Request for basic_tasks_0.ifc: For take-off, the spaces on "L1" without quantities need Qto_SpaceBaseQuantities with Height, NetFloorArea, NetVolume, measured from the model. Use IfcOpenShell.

First a look at what the model holds.

```python
import ifcopenshell
import ifcopenshell.util.element
import ifcopenshell.util.unit

model = ifcopenshell.open("basic_tasks_0.ifc")
print(model.schema)
for unit_type in ("LENGTHUNIT", "AREAUNIT", "VOLUMEUNIT"):
    print(unit_type, ifcopenshell.util.unit.calculate_unit_scale(model, unit_type))
storey = next(s for s in model.by_type("IfcBuildingStorey") if s.Name == "L1")
spaces = [e for e in ifcopenshell.util.element.get_decomposition(storey) if e.is_a("IfcSpace")]
for e in sorted(spaces, key=lambda e: e.id()):
    print(e.id(), e.is_a(), e.Name, list(ifcopenshell.util.element.get_psets(e, qtos_only=True)), sep=" | ")
```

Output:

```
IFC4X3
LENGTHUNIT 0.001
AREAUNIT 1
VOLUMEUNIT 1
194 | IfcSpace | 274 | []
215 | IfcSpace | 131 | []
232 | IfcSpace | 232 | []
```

```python
import ifcopenshell
import ifcopenshell.api.pset
import ifcopenshell.geom
import ifcopenshell.util.element
import ifcopenshell.util.shape
import ifcopenshell.util.unit

model = ifcopenshell.open("basic_tasks_0.ifc")
unit_scale = ifcopenshell.util.unit.calculate_unit_scale(model)
area_scale = ifcopenshell.util.unit.calculate_unit_scale(model, "AREAUNIT")
volume_scale = ifcopenshell.util.unit.calculate_unit_scale(model, "VOLUMEUNIT")
settings = ifcopenshell.geom.settings()

storey = next(s for s in model.by_type("IfcBuildingStorey") if s.Name == "L1")
spaces = [e for e in ifcopenshell.util.element.get_decomposition(storey) if e.is_a("IfcSpace")]

for e in sorted(spaces, key=lambda e: e.id()):
    if ifcopenshell.util.element.get_psets(e, qtos_only=True, should_inherit=False):
        continue
    # Geometry comes back in metres, in the element's own axes.
    shape = ifcopenshell.geom.create_shape(settings, e)
    values = {
        "Height": ifcopenshell.util.shape.get_z(shape.geometry) / unit_scale,
        "NetFloorArea": ifcopenshell.util.shape.get_footprint_area(shape.geometry) / area_scale,
        "NetVolume": ifcopenshell.util.shape.get_volume(shape.geometry) / volume_scale,
    }
    qto = ifcopenshell.api.pset.add_qto(model, product=e, name="Qto_SpaceBaseQuantities")
    ifcopenshell.api.pset.edit_qto(model, qto=qto, properties=values)
    print(e.id(), {k: round(v, 3) for k, v in values.items()})

model.write("basic_tasks_0-out.ifc")
```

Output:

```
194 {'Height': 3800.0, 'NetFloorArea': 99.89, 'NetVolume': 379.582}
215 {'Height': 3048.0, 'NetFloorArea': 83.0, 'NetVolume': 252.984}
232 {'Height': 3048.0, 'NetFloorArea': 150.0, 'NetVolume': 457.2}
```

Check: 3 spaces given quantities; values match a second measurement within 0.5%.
